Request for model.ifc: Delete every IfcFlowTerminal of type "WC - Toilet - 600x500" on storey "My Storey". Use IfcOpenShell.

First a look at what the model holds.

```python
import ifcopenshell
import ifcopenshell.util.element

model = ifcopenshell.open("model.ifc")
print(model.schema)
storey = next(s for s in model.by_type("IfcBuildingStorey") if s.Name == "My Storey")
terminals = [e for e in ifcopenshell.util.element.get_decomposition(storey) if e.is_a("IfcFlowTerminal")]
seen = {}
for e in terminals:
    element_type = ifcopenshell.util.element.get_type(e)
    name = element_type.Name if element_type not in (None, e) else None
    seen[name] = seen.get(name, 0) + 1
for name, count in sorted(seen.items(), key=str):
    print(count, "x", name)
```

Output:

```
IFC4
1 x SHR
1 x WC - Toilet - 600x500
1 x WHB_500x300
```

```python
import ifcopenshell
import ifcopenshell.api.root
import ifcopenshell.util.element

model = ifcopenshell.open("model.ifc")

storey = next(s for s in model.by_type("IfcBuildingStorey") if s.Name == "My Storey")
terminals = [e for e in ifcopenshell.util.element.get_decomposition(storey) if e.is_a("IfcFlowTerminal")]
targets = [e for e in terminals if (t := ifcopenshell.util.element.get_type(e)) not in (None, e) and t.Name == "WC - Toilet - 600x500"]

for e in targets:
    ifcopenshell.api.root.remove_product(model, product=e)
print(len(targets), "removed")

model.write("model_v2.ifc")
```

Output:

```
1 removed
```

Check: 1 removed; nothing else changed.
